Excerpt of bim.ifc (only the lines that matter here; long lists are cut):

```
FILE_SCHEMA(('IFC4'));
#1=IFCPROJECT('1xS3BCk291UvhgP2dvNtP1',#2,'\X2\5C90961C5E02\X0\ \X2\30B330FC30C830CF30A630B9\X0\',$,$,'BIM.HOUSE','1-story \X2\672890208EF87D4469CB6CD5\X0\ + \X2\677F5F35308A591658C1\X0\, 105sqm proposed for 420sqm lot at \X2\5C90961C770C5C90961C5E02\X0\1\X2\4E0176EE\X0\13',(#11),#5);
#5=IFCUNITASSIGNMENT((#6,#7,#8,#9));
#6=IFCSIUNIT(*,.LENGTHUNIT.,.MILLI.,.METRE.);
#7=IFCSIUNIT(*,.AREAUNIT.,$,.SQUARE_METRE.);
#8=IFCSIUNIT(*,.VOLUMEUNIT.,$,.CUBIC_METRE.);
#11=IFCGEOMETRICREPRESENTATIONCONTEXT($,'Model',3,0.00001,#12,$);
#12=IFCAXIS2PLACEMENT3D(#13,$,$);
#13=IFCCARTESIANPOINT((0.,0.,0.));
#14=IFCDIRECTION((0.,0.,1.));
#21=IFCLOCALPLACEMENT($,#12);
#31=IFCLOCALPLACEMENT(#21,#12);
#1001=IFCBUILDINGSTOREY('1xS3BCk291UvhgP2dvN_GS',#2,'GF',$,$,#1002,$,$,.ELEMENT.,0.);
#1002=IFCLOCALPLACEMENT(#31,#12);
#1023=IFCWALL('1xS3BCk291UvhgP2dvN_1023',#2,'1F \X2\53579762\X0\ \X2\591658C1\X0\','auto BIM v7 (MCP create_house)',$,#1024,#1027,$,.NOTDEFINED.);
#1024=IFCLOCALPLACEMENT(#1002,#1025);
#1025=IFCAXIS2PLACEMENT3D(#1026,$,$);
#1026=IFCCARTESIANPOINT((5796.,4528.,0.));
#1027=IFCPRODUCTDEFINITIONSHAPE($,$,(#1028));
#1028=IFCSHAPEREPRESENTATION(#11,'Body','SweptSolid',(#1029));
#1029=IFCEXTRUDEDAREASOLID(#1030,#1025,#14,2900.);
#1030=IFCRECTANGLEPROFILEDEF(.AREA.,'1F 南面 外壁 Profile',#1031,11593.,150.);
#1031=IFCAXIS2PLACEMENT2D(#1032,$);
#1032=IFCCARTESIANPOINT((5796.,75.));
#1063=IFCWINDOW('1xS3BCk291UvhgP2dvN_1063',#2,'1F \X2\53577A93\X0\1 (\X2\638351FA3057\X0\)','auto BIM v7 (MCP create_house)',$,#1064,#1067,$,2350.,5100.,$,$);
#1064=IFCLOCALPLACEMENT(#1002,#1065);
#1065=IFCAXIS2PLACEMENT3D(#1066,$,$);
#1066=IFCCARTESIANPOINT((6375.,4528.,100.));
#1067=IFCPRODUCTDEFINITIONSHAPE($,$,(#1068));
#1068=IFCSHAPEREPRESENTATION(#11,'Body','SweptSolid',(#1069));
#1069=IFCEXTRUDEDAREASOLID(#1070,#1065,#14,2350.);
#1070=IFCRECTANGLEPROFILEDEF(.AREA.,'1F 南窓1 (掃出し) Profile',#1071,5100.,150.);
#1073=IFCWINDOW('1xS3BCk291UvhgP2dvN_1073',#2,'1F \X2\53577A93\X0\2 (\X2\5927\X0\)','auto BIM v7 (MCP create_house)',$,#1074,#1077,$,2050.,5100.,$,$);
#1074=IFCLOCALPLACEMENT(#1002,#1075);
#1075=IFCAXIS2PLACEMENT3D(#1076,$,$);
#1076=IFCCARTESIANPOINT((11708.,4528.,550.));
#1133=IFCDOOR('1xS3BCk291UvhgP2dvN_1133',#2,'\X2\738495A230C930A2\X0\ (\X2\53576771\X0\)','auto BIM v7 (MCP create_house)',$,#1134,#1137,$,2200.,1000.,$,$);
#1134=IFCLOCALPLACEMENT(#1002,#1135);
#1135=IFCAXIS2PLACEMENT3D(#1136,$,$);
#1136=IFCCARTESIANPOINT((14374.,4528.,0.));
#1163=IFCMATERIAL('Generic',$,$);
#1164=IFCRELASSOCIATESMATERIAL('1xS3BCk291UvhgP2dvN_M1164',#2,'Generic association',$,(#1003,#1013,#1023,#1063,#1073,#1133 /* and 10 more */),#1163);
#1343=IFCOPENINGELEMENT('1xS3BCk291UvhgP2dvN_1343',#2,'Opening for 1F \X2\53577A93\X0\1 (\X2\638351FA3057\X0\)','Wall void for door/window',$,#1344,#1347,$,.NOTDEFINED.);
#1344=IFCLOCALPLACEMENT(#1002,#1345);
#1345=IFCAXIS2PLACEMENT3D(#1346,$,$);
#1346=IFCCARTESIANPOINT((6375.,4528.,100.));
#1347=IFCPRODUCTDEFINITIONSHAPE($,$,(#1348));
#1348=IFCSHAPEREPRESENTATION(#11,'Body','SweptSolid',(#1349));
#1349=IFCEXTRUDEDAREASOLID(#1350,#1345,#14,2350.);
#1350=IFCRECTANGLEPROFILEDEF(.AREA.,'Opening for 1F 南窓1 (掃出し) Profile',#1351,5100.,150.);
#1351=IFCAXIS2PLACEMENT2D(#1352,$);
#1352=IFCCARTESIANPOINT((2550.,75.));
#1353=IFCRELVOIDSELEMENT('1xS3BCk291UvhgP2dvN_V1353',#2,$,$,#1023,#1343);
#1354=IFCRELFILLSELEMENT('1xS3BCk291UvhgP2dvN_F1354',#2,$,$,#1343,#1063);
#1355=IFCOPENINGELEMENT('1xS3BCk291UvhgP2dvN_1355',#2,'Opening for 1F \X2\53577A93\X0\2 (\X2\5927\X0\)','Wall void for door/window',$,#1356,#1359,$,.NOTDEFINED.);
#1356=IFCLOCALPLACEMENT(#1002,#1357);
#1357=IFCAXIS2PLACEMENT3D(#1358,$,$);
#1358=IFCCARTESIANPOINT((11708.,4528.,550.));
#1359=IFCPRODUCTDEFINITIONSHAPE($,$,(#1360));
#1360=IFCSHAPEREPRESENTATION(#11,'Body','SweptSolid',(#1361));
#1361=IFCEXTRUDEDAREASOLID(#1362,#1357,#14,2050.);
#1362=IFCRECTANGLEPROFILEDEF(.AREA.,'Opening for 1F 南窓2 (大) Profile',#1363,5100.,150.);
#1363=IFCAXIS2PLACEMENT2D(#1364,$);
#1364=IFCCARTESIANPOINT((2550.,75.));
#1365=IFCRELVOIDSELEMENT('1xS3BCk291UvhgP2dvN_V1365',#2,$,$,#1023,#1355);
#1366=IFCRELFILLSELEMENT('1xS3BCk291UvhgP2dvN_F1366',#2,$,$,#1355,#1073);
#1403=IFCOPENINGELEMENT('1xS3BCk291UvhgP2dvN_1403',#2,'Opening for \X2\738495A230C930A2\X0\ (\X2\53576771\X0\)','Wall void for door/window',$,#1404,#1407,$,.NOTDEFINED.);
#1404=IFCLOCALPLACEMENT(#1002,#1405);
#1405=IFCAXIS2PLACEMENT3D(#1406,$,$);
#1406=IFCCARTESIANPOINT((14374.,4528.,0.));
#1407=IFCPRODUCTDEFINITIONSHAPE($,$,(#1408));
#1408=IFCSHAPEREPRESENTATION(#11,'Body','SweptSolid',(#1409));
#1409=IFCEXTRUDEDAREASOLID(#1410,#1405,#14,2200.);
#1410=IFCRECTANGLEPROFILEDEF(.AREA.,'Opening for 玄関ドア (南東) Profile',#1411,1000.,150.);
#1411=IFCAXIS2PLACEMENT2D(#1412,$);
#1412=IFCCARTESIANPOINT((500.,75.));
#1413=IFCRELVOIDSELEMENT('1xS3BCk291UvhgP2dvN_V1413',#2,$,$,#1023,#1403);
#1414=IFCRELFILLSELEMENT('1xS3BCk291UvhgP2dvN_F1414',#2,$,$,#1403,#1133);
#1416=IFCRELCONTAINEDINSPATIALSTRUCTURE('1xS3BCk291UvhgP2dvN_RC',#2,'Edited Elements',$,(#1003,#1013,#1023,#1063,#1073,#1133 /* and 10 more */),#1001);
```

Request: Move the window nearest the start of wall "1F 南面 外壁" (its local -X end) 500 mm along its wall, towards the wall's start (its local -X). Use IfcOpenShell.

```python
import ifcopenshell
import ifcopenshell.api.geometry
import ifcopenshell.util.placement
import ifcopenshell.util.unit

model = ifcopenshell.open("bim.ifc")
unit_scale = ifcopenshell.util.unit.calculate_unit_scale(model)

window = model.by_id(1063)
opening = window.FillsVoids[0].RelatingOpeningElement
wall = opening.VoidsElements[0].RelatingBuildingElement

wall_matrix = ifcopenshell.util.placement.get_local_placement(wall.ObjectPlacement)
shift = wall_matrix[:3, 0] * -0.5 / unit_scale
before = ifcopenshell.util.placement.get_local_placement(window.ObjectPlacement)[:3, 3].copy()

# The window is not placed relative to its opening, so move both.
for product in (opening, window):
    matrix = ifcopenshell.util.placement.get_local_placement(product.ObjectPlacement)
    matrix[:3, 3] += shift
    ifcopenshell.api.geometry.edit_object_placement(model, product=product, matrix=matrix, is_si=False)

after = ifcopenshell.util.placement.get_local_placement(window.ObjectPlacement)[:3, 3]
print("window moved by", (after - before).round(3) + 0.0)

model.write("bim_v2.ifc")
```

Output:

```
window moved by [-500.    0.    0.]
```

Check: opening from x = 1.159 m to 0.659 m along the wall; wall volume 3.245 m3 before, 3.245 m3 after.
